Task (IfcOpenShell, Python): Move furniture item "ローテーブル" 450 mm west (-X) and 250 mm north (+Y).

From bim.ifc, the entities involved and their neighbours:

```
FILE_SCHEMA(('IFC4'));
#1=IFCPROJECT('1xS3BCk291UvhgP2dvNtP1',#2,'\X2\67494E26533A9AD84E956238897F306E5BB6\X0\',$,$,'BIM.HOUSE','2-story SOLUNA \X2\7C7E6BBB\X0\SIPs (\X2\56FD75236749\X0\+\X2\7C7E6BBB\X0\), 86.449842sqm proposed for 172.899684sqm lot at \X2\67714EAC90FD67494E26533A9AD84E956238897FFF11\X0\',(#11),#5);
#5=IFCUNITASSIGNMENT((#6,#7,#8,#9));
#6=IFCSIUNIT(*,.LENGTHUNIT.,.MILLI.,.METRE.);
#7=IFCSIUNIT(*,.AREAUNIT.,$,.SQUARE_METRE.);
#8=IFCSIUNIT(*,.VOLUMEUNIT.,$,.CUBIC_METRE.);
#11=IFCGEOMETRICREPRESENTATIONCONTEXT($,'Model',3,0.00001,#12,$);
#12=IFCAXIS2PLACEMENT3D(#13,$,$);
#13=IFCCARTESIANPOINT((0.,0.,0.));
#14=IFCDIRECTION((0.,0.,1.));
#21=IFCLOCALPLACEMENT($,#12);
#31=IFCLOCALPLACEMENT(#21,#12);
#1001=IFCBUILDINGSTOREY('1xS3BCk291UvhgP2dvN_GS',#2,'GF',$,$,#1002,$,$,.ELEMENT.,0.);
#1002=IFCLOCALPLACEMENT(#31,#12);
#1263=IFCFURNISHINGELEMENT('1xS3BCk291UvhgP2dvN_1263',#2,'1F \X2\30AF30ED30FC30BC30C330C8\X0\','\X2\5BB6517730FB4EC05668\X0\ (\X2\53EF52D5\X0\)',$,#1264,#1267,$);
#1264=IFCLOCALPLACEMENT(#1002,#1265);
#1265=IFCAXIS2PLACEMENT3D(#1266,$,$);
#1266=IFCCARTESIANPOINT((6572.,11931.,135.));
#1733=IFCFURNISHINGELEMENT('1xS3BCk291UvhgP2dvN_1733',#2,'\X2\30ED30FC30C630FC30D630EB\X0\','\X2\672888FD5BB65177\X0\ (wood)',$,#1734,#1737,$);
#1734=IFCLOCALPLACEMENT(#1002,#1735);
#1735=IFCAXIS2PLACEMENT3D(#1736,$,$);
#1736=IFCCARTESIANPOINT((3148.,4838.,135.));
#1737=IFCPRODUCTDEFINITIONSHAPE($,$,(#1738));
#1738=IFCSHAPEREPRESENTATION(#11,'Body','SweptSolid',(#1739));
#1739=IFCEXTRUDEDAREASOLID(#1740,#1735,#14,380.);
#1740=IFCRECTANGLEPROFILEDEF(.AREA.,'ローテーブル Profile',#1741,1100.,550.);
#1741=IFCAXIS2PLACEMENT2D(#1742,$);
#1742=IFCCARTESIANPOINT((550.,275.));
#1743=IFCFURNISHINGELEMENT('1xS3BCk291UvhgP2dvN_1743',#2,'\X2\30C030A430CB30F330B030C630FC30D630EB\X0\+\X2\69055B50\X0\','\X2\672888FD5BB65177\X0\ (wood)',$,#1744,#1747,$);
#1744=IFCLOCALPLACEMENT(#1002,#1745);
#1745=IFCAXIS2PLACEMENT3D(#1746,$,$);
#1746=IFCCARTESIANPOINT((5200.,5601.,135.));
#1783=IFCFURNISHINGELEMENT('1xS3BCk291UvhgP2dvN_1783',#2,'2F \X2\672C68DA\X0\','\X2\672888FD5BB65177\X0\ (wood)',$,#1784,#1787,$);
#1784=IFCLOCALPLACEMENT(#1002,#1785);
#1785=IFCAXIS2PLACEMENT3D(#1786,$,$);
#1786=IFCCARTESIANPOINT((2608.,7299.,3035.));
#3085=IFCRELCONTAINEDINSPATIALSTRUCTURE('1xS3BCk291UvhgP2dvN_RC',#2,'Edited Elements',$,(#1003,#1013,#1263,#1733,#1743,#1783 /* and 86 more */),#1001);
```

```python
import ifcopenshell
import ifcopenshell.api.geometry
import ifcopenshell.util.placement
import ifcopenshell.util.unit

model = ifcopenshell.open("bim.ifc")
unit_scale = ifcopenshell.util.unit.calculate_unit_scale(model)

item = model.by_guid("1xS3BCk291UvhgP2dvN_1733")
matrix = ifcopenshell.util.placement.get_local_placement(item.ObjectPlacement)
matrix[0, 3] -= 0.45 / unit_scale
matrix[1, 3] += 0.25 / unit_scale
ifcopenshell.api.geometry.edit_object_placement(model, product=item, matrix=matrix, is_si=False)

print(ifcopenshell.util.placement.get_local_placement(item.ObjectPlacement).round(3) + 0.0)

model.write("bim-out.ifc")
```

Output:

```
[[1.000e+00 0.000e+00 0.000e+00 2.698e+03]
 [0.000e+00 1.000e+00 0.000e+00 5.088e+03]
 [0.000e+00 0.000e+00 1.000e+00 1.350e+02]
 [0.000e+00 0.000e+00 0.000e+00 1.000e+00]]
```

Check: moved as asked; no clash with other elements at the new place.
